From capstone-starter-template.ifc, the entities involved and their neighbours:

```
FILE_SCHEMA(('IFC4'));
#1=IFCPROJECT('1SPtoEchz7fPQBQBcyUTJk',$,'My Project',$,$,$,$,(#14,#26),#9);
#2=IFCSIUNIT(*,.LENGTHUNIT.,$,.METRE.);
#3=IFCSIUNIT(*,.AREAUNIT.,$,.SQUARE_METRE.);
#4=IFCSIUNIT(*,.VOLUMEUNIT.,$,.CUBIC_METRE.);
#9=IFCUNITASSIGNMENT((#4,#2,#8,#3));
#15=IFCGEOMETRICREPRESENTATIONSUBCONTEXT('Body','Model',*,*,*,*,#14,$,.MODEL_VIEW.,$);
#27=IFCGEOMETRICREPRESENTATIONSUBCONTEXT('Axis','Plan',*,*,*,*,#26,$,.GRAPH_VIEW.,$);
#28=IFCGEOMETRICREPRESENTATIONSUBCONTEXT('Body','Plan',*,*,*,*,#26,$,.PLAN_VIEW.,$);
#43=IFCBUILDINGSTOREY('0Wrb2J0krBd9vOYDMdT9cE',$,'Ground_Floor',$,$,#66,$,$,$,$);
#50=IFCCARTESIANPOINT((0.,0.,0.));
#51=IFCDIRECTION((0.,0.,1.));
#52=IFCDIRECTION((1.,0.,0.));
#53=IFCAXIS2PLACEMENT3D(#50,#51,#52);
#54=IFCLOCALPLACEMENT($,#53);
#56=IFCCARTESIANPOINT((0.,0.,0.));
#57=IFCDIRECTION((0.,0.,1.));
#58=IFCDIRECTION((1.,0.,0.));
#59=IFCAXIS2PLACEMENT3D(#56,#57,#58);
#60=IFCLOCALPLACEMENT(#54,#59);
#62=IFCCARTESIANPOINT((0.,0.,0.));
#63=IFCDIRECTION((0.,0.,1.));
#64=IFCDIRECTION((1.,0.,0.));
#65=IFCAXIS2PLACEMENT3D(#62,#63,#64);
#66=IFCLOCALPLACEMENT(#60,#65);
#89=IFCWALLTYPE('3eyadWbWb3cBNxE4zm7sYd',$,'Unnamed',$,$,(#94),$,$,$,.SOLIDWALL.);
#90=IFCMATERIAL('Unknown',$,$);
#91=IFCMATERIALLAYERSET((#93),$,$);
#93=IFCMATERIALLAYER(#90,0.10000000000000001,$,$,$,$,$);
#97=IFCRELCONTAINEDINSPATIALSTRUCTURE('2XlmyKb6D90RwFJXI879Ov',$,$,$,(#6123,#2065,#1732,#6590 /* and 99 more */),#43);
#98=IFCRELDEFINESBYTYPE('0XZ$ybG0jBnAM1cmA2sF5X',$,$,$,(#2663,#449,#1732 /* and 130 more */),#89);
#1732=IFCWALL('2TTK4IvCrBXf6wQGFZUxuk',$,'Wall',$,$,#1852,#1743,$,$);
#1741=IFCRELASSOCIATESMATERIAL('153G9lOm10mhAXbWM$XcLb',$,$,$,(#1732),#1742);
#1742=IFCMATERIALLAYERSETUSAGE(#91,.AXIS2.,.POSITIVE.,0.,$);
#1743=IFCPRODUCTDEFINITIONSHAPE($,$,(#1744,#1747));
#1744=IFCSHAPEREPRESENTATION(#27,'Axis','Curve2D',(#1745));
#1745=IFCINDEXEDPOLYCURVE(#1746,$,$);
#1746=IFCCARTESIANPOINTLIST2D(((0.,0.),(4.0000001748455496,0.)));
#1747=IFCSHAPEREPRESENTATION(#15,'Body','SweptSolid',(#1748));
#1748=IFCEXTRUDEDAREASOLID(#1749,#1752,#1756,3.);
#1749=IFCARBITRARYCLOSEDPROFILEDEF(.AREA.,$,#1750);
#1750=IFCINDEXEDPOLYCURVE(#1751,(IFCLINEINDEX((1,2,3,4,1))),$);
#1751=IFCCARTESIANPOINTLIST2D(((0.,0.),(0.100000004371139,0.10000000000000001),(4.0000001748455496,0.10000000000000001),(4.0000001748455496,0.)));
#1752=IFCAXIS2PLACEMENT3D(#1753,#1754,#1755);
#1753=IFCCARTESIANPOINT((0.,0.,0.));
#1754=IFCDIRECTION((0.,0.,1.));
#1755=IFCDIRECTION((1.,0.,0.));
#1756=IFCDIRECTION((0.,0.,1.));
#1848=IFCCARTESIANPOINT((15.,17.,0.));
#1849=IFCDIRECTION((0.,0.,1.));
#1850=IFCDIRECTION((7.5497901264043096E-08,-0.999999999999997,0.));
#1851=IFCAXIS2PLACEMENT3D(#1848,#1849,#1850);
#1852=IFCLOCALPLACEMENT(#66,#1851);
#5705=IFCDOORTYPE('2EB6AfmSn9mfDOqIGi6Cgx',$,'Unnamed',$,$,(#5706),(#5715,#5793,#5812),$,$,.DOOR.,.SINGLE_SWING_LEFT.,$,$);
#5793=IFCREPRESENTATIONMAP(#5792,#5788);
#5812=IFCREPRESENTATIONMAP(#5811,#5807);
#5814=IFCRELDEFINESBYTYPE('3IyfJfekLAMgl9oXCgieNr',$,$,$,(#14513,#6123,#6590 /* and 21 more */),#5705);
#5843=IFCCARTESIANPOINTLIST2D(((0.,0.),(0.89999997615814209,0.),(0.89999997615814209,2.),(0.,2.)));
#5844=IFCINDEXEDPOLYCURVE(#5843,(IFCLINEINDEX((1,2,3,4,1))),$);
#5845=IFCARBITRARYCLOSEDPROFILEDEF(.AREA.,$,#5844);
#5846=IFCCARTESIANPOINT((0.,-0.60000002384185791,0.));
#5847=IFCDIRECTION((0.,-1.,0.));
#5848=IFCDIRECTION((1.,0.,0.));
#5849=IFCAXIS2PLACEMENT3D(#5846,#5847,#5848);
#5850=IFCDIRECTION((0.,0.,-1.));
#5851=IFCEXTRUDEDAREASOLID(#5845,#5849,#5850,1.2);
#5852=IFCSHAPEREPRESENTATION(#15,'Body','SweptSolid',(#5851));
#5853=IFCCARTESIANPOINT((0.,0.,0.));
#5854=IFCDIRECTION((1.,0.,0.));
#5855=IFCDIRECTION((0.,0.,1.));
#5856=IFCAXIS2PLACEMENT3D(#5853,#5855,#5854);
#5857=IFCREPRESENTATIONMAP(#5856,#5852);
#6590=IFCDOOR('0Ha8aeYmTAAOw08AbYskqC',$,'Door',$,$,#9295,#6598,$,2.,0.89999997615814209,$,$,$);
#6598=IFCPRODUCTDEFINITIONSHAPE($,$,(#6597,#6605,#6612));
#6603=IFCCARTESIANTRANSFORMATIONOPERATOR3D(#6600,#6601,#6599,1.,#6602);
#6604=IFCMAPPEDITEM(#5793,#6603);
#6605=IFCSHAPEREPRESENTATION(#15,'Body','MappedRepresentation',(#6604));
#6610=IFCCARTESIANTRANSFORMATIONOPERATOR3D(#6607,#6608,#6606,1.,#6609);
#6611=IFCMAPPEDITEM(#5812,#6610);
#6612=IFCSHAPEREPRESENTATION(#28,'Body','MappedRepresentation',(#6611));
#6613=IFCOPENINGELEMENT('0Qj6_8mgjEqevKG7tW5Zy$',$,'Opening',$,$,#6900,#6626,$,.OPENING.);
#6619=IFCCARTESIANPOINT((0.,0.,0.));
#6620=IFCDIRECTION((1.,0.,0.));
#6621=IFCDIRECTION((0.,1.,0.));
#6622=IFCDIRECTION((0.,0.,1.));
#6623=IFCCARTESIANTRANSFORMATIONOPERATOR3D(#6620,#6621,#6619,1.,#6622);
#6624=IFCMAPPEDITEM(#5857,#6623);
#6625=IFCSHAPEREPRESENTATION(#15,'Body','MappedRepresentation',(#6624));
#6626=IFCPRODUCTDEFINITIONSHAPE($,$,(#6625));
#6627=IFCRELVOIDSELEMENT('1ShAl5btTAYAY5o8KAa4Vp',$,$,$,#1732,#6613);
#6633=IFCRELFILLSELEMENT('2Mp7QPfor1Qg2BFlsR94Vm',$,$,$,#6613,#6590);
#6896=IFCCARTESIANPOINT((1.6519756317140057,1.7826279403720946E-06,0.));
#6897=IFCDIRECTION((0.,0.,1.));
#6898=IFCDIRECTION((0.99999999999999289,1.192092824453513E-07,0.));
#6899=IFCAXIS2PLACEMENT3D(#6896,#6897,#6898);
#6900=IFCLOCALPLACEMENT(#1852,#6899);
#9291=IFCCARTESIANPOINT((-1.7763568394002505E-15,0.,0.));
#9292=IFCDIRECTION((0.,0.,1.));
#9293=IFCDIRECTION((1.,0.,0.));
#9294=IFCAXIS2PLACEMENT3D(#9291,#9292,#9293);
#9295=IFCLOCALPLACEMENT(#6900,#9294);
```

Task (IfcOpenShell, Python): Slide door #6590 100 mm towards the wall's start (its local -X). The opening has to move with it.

```python
import ifcopenshell
import ifcopenshell.api.geometry
import ifcopenshell.util.placement

model = ifcopenshell.open("capstone-starter-template.ifc")

door = model.by_guid("0Ha8aeYmTAAOw08AbYskqC")
opening = door.FillsVoids[0].RelatingOpeningElement
wall = opening.VoidsElements[0].RelatingBuildingElement

wall_matrix = ifcopenshell.util.placement.get_local_placement(wall.ObjectPlacement)
shift = wall_matrix[:3, 0] * -0.1
before = ifcopenshell.util.placement.get_local_placement(door.ObjectPlacement)[:3, 3].copy()

# The door is placed relative to its opening, so it follows when the opening moves.
matrix = ifcopenshell.util.placement.get_local_placement(opening.ObjectPlacement)
matrix[:3, 3] += shift
ifcopenshell.api.geometry.edit_object_placement(
    model, product=opening, matrix=matrix, is_si=False, should_transform_children=True
)

after = ifcopenshell.util.placement.get_local_placement(door.ObjectPlacement)[:3, 3]
print("door moved by", (after - before).round(3) + 0.0)

model.write("capstone-starter-template_updated.ifc")
```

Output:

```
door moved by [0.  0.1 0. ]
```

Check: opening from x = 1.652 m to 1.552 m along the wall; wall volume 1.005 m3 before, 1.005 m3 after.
